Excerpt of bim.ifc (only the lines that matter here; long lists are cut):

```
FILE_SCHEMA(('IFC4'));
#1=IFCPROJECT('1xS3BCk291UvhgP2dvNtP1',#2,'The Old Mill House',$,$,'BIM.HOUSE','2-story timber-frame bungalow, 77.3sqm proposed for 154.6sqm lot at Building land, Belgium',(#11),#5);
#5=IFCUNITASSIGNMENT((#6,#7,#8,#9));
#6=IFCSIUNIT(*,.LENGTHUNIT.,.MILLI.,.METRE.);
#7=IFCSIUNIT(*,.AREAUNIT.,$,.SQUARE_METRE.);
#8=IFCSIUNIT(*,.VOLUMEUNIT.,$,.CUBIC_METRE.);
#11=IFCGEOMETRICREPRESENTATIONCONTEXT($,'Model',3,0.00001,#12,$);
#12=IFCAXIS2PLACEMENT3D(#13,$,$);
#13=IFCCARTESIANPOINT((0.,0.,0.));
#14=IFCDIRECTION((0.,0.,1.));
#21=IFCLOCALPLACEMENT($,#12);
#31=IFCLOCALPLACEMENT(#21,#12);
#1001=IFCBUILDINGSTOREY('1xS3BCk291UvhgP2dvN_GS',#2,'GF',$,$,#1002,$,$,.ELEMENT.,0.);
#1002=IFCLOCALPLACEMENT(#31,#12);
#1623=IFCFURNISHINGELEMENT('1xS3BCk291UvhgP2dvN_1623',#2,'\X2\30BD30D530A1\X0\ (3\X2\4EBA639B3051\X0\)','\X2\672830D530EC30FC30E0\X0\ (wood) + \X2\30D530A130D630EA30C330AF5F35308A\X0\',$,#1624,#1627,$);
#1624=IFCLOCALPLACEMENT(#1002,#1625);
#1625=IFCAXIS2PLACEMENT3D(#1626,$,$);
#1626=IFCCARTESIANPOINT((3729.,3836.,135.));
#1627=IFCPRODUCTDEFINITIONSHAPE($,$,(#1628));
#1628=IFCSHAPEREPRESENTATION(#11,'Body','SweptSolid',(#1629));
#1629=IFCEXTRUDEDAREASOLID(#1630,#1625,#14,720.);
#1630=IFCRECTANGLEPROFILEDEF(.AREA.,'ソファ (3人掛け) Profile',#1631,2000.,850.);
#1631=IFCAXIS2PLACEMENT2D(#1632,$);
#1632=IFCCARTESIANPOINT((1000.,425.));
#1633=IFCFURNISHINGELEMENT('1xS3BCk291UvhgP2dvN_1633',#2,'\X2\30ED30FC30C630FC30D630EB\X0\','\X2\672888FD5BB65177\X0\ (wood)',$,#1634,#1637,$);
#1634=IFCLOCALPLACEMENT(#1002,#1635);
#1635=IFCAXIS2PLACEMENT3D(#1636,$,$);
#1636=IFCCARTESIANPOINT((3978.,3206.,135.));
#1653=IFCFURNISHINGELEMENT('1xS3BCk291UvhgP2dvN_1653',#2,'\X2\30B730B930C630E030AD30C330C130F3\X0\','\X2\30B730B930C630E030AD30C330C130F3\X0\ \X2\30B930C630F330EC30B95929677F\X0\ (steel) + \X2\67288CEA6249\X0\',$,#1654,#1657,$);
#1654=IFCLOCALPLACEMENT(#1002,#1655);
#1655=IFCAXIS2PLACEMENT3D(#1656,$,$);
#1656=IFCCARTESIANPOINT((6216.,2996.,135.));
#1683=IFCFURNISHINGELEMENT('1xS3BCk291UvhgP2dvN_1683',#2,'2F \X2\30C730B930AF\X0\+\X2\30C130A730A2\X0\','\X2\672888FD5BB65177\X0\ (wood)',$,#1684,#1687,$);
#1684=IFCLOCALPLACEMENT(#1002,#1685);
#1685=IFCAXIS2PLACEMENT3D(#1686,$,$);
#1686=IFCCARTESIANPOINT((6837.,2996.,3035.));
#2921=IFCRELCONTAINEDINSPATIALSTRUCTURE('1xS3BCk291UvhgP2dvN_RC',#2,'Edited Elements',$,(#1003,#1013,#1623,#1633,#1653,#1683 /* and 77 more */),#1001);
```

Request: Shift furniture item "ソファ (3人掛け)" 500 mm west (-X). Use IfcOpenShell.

```python
import ifcopenshell
import ifcopenshell.api.geometry
import ifcopenshell.util.placement

model = ifcopenshell.open("bim.ifc")

item = model.by_id(1623)
matrix = ifcopenshell.util.placement.get_local_placement(item.ObjectPlacement)
matrix[0, 3] -= 500.0
ifcopenshell.api.geometry.edit_object_placement(model, product=item, matrix=matrix, is_si=False)

print(ifcopenshell.util.placement.get_local_placement(item.ObjectPlacement).round(3) + 0.0)

model.write("bim_edited.ifc")
```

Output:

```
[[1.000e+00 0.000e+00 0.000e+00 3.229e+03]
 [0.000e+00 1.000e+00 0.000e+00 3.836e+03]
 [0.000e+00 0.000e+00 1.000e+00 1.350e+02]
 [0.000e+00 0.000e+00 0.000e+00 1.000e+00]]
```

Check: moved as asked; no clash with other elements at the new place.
